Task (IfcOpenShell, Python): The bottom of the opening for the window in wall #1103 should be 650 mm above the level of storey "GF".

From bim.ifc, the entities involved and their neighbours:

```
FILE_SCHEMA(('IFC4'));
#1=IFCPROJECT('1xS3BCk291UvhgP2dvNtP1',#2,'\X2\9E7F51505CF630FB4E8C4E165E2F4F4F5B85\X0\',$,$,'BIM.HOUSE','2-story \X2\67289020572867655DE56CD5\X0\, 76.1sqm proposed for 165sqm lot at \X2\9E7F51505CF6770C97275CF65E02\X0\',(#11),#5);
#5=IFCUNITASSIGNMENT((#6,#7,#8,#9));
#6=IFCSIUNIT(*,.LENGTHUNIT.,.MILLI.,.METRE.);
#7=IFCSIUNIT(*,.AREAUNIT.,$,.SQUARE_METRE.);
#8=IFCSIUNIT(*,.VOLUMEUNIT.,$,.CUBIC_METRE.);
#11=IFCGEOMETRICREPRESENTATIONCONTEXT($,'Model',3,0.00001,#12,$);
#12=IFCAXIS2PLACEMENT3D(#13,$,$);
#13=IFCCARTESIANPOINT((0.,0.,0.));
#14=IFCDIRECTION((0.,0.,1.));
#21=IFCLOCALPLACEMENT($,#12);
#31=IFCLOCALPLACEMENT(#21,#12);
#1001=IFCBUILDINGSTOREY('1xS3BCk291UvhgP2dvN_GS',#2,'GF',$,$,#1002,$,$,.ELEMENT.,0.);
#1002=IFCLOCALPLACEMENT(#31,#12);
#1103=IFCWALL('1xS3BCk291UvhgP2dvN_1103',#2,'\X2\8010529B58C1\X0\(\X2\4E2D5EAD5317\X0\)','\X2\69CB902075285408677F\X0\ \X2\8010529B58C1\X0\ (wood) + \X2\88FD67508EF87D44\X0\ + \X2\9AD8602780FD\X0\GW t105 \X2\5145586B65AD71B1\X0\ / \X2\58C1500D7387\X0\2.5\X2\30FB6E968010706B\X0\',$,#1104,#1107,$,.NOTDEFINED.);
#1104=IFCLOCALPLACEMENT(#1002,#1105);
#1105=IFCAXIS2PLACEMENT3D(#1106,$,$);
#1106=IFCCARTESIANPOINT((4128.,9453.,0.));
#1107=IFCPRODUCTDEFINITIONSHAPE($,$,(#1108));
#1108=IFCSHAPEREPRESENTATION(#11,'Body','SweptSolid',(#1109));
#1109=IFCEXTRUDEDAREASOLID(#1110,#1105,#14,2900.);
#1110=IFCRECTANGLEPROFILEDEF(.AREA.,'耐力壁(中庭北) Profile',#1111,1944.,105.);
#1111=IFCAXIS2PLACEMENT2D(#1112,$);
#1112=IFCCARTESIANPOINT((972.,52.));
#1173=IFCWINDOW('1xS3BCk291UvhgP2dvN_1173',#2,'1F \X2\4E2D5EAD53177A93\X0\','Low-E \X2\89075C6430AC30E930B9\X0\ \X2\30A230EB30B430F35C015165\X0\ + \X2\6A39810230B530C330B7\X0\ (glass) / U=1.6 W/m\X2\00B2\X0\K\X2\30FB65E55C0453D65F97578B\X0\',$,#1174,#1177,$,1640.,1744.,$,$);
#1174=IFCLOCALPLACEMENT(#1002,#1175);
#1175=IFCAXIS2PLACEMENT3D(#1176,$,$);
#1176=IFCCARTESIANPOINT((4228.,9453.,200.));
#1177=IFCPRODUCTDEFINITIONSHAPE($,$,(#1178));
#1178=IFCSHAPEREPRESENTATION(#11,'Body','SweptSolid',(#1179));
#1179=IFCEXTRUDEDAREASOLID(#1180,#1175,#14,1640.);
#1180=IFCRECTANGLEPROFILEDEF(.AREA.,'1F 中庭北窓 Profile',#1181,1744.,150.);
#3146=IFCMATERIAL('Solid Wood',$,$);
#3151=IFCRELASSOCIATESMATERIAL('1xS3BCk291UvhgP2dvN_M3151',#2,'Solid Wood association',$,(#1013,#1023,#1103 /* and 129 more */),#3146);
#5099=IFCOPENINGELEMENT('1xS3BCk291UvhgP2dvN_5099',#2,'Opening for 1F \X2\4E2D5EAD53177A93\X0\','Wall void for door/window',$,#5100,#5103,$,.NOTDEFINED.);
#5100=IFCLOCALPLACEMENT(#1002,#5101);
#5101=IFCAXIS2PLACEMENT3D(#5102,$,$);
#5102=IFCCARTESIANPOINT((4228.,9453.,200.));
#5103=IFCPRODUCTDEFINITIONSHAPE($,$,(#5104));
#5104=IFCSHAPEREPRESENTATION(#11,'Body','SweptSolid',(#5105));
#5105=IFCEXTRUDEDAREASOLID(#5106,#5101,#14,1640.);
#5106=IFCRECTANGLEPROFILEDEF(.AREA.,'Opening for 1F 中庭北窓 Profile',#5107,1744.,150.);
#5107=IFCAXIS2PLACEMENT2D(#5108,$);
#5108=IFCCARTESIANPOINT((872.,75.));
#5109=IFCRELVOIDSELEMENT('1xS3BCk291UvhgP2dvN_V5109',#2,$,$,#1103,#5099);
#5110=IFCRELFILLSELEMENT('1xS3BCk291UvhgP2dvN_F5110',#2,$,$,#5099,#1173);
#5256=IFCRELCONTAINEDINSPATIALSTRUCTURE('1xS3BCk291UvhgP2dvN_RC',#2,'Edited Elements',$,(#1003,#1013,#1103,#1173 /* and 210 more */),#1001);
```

```python
import numpy as np
import ifcopenshell
import ifcopenshell.api.geometry
import ifcopenshell.geom
import ifcopenshell.util.element
import ifcopenshell.util.placement
import ifcopenshell.util.shape
import ifcopenshell.util.unit

model = ifcopenshell.open("bim.ifc")
unit_scale = ifcopenshell.util.unit.calculate_unit_scale(model)

window = model.by_id(1173)
opening = window.FillsVoids[0].RelatingOpeningElement
storey = ifcopenshell.util.element.get_container(window, ifc_class="IfcBuildingStorey")
level = ifcopenshell.util.placement.get_local_placement(storey.ObjectPlacement)[2, 3]

# The opening's origin need not be at the sill, so measure its lowest point.
shape = ifcopenshell.geom.create_shape(ifcopenshell.geom.settings(), opening)
bottom = ifcopenshell.util.shape.get_shape_bottom_elevation(shape, shape.geometry) / unit_scale
dz = level + 0.65 / unit_scale - bottom

shift = np.array([0.0, 0.0, dz])
# The window is not placed relative to its opening, so move both.
for product in (opening, window):
    matrix = ifcopenshell.util.placement.get_local_placement(product.ObjectPlacement)
    matrix[:3, 3] += shift
    ifcopenshell.api.geometry.edit_object_placement(model, product=product, matrix=matrix, is_si=False)

print(f"moved by {dz * unit_scale:+.3f} m")

model.write("bim_v2.ifc")
```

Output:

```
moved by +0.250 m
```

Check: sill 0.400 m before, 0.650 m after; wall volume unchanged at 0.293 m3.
